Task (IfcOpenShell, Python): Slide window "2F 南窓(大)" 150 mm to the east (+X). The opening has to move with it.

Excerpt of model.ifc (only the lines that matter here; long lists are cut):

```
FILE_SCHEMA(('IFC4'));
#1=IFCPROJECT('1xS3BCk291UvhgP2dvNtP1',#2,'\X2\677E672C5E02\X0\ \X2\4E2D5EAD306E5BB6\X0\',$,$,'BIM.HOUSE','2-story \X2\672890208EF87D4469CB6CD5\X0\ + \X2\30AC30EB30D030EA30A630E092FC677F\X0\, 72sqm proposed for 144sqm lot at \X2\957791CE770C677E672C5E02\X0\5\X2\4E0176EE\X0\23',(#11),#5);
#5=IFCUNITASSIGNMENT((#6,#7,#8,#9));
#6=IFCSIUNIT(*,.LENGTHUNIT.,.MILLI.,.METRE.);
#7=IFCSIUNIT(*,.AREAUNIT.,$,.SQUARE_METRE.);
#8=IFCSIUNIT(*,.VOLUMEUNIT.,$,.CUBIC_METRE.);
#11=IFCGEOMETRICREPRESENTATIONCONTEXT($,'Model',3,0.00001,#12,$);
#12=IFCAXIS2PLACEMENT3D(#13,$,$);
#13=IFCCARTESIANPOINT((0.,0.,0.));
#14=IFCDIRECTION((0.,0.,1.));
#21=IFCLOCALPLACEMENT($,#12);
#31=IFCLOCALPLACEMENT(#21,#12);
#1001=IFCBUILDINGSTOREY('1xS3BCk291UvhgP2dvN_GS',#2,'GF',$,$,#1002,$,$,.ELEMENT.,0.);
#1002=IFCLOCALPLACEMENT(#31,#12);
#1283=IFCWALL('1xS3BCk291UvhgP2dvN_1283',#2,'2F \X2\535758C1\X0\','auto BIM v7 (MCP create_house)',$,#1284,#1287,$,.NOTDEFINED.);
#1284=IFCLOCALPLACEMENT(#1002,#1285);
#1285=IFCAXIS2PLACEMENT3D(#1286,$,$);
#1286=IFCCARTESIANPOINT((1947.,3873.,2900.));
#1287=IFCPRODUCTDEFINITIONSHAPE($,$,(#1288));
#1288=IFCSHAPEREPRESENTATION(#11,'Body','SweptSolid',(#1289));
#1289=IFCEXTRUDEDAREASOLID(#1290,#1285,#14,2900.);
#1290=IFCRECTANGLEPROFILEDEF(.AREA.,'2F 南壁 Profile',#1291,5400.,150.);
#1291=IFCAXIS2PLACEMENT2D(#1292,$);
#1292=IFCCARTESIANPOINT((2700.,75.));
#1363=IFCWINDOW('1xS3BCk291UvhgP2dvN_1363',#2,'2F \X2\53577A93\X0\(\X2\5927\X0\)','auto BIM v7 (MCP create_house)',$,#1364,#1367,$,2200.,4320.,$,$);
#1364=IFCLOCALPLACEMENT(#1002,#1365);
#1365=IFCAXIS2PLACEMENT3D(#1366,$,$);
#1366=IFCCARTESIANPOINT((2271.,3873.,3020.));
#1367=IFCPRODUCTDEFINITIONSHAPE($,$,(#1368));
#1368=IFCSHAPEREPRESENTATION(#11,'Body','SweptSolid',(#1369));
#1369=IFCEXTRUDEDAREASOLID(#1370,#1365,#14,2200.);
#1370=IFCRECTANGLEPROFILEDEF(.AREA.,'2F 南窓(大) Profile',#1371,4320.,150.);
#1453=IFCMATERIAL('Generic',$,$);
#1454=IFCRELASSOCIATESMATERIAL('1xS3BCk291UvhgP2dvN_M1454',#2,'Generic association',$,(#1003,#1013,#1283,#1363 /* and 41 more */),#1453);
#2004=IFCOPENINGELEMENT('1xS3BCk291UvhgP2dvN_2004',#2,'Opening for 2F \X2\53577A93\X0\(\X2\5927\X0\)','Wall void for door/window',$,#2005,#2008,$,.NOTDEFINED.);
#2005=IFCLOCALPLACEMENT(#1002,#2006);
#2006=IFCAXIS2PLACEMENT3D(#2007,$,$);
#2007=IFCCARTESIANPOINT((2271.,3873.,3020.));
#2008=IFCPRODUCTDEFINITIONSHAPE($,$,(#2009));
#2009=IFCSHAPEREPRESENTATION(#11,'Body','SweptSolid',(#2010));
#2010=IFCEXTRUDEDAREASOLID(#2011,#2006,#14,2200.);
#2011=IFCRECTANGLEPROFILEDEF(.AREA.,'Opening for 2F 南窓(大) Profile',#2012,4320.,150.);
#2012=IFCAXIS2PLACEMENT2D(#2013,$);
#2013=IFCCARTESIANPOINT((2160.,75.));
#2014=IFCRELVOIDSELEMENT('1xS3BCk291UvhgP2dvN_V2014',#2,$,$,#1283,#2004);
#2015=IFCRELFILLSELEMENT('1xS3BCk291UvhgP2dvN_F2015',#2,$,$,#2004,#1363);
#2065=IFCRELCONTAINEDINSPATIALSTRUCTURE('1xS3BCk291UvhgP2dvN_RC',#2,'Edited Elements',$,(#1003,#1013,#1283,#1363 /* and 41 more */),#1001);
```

```python
import ifcopenshell
import ifcopenshell.api.geometry
import ifcopenshell.util.placement

model = ifcopenshell.open("model.ifc")

window = model.by_guid("1xS3BCk291UvhgP2dvN_1363")
opening = window.FillsVoids[0].RelatingOpeningElement
wall = opening.VoidsElements[0].RelatingBuildingElement

wall_matrix = ifcopenshell.util.placement.get_local_placement(wall.ObjectPlacement)
shift = wall_matrix[:3, 0] * 150.0
before = ifcopenshell.util.placement.get_local_placement(window.ObjectPlacement)[:3, 3].copy()

# The window is not placed relative to its opening, so move both.
for product in (opening, window):
    matrix = ifcopenshell.util.placement.get_local_placement(product.ObjectPlacement)
    matrix[:3, 3] += shift
    ifcopenshell.api.geometry.edit_object_placement(model, product=product, matrix=matrix, is_si=False)

after = ifcopenshell.util.placement.get_local_placement(window.ObjectPlacement)[:3, 3]
print("window moved by", (after - before).round(3) + 0.0)

model.write("model_rev.ifc")
```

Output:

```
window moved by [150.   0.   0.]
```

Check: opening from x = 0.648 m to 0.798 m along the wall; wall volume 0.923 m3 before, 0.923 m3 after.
